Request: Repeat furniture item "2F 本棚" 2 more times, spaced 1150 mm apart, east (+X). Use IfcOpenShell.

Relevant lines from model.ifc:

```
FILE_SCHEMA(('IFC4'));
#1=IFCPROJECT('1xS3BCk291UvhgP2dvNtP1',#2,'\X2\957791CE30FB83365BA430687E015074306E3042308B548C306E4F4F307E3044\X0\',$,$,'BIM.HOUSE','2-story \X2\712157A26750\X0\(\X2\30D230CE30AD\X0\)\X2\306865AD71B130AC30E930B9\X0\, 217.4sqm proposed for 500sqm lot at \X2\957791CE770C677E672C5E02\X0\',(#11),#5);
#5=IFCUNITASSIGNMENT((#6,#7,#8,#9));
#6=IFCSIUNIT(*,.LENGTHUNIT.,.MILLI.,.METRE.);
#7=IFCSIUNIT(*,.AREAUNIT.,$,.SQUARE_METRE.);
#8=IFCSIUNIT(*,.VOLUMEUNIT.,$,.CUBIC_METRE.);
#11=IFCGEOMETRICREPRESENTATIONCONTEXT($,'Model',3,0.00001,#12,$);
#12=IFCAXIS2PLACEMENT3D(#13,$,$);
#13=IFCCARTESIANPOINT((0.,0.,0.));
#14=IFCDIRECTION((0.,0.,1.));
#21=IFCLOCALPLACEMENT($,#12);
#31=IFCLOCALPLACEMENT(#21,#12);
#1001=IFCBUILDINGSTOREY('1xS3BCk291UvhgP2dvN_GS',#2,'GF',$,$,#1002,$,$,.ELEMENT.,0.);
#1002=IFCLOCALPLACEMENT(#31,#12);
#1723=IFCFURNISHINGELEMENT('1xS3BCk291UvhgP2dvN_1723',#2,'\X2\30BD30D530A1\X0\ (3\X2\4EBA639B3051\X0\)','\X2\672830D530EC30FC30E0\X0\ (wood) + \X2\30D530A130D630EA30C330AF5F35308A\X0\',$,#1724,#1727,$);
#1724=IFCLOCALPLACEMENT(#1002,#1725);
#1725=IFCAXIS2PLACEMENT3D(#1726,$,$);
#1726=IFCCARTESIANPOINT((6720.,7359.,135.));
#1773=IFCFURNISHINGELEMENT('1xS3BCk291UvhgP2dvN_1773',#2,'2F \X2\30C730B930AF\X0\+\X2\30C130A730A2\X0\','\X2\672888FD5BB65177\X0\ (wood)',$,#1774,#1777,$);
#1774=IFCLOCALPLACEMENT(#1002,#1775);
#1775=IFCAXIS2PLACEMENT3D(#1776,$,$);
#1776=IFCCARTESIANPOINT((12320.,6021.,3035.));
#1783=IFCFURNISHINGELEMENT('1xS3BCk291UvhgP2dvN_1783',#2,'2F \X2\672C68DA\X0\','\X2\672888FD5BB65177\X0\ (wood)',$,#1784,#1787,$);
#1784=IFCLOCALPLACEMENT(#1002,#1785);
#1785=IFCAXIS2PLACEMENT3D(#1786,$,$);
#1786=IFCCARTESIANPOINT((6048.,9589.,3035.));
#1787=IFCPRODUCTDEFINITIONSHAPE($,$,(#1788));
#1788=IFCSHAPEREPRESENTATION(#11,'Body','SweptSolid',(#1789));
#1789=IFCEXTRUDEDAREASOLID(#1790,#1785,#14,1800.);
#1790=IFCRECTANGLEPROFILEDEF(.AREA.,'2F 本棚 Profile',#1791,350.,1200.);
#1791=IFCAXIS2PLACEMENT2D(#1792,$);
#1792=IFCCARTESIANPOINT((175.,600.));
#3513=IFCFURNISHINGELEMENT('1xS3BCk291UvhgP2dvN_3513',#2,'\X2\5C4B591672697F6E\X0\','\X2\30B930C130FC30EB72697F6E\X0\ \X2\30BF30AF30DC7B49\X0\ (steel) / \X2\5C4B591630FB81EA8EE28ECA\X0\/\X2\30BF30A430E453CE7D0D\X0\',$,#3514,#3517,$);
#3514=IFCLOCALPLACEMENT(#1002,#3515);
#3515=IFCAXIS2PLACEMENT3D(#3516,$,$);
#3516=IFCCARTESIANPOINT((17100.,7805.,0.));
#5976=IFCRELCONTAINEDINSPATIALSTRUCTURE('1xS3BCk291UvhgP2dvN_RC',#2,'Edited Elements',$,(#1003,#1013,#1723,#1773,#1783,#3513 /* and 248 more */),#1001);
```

```python
import numpy as np
import ifcopenshell
import ifcopenshell.api.geometry
import ifcopenshell.api.root
import ifcopenshell.util.element
import ifcopenshell.util.placement

model = ifcopenshell.open("model.ifc")


def reuse_history(source, copy):
    """copy_class also copies each property set's owner history, people and application; keep the originals."""
    for rel in copy.IsDefinedBy:
        if rel.is_a("IfcRelDefinesByProperties") and (history := rel.RelatingPropertyDefinition.OwnerHistory):
            rel.RelatingPropertyDefinition.OwnerHistory = source.OwnerHistory
            ifcopenshell.util.element.remove_deep2(model, history)


source = model.by_id(1783)
base = ifcopenshell.util.placement.get_local_placement(source.ObjectPlacement)
step = np.array([1.0, 0.0, 0.0]) * 1150.0

for i in range(1, 3):
    copy = ifcopenshell.api.root.copy_class(model, product=source)
    copy.Representation = ifcopenshell.util.element.copy_deep(
        model, source.Representation, exclude=["IfcGeometricRepresentationContext", "IfcRepresentationMap"]
    )
    reuse_history(source, copy)
    matrix = base.copy()
    matrix[:3, 3] += i * step
    print("added at", matrix[:3, 3].round(3) + 0.0)
    ifcopenshell.api.geometry.edit_object_placement(model, product=copy, matrix=matrix, is_si=False)

model.write("model-out.ifc")
```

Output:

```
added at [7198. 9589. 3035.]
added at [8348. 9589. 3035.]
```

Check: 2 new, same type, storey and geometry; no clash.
